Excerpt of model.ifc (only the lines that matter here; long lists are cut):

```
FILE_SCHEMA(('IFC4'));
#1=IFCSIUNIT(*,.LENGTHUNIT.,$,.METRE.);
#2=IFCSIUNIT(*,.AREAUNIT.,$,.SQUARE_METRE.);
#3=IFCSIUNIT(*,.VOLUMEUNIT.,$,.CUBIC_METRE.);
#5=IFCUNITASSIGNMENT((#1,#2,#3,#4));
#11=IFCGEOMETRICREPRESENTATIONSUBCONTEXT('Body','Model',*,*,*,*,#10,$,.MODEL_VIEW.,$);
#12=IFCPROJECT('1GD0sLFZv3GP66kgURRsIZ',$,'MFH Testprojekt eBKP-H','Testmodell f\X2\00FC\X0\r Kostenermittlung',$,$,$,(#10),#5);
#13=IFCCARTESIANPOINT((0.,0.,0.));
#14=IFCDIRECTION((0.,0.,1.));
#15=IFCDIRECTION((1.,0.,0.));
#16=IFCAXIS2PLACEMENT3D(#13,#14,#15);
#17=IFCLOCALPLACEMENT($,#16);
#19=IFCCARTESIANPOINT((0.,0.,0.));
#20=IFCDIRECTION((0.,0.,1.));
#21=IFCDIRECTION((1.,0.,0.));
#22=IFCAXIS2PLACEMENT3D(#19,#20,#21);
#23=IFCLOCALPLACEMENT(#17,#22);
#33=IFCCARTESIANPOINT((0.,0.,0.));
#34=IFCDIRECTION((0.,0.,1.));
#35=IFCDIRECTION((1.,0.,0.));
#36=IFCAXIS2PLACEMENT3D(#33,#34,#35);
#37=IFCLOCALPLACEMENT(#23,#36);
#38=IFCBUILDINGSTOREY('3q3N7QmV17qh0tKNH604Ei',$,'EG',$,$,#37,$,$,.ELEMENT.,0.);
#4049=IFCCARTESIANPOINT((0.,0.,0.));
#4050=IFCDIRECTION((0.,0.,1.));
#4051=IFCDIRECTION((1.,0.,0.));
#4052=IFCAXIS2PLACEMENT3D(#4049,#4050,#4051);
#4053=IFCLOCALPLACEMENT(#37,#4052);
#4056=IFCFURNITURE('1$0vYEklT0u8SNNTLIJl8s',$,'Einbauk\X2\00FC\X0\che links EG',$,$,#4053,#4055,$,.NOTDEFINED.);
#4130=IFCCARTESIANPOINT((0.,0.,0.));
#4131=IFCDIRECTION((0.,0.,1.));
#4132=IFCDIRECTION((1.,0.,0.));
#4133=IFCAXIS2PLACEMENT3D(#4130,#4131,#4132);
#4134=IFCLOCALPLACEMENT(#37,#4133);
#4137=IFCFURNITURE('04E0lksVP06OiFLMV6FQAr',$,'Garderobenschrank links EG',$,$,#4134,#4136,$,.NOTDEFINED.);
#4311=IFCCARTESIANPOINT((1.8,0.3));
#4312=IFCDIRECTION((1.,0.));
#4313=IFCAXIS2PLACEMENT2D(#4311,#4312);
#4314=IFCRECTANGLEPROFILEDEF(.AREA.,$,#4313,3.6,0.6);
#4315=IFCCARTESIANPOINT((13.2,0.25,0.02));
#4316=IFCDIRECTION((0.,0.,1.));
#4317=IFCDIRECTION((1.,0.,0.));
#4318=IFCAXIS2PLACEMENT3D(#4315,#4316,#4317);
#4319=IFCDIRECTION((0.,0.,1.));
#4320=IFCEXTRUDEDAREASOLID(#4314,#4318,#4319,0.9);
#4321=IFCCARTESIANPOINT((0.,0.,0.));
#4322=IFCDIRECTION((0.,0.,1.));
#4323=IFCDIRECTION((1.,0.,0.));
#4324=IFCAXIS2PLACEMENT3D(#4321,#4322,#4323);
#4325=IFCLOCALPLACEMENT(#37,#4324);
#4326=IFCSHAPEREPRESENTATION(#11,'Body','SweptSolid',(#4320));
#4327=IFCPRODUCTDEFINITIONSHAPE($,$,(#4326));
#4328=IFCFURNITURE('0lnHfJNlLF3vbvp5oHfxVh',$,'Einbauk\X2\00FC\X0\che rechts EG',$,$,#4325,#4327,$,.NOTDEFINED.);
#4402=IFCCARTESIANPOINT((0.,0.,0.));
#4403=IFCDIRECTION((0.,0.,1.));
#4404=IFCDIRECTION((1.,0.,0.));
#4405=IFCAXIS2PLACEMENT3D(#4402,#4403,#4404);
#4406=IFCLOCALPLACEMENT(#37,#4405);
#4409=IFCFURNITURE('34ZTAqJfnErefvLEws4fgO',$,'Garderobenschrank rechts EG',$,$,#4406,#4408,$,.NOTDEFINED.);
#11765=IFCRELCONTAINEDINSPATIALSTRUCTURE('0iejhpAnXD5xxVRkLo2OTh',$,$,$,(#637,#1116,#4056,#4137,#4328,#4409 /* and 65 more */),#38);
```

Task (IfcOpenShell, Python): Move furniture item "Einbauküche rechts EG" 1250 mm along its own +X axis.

```python
import ifcopenshell
import ifcopenshell.api.geometry
import ifcopenshell.util.placement
import ifcopenshell.util.unit

model = ifcopenshell.open("model.ifc")
unit_scale = ifcopenshell.util.unit.calculate_unit_scale(model)

item = model.by_id(4328)
matrix = ifcopenshell.util.placement.get_local_placement(item.ObjectPlacement)
matrix[:3, 3] += matrix[:3, 0] * 1.25 / unit_scale
ifcopenshell.api.geometry.edit_object_placement(model, product=item, matrix=matrix, is_si=False)

print(ifcopenshell.util.placement.get_local_placement(item.ObjectPlacement).round(3) + 0.0)

model.write("model_edited.ifc")
```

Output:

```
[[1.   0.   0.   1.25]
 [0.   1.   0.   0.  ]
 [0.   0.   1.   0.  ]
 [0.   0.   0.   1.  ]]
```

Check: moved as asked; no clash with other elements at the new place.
